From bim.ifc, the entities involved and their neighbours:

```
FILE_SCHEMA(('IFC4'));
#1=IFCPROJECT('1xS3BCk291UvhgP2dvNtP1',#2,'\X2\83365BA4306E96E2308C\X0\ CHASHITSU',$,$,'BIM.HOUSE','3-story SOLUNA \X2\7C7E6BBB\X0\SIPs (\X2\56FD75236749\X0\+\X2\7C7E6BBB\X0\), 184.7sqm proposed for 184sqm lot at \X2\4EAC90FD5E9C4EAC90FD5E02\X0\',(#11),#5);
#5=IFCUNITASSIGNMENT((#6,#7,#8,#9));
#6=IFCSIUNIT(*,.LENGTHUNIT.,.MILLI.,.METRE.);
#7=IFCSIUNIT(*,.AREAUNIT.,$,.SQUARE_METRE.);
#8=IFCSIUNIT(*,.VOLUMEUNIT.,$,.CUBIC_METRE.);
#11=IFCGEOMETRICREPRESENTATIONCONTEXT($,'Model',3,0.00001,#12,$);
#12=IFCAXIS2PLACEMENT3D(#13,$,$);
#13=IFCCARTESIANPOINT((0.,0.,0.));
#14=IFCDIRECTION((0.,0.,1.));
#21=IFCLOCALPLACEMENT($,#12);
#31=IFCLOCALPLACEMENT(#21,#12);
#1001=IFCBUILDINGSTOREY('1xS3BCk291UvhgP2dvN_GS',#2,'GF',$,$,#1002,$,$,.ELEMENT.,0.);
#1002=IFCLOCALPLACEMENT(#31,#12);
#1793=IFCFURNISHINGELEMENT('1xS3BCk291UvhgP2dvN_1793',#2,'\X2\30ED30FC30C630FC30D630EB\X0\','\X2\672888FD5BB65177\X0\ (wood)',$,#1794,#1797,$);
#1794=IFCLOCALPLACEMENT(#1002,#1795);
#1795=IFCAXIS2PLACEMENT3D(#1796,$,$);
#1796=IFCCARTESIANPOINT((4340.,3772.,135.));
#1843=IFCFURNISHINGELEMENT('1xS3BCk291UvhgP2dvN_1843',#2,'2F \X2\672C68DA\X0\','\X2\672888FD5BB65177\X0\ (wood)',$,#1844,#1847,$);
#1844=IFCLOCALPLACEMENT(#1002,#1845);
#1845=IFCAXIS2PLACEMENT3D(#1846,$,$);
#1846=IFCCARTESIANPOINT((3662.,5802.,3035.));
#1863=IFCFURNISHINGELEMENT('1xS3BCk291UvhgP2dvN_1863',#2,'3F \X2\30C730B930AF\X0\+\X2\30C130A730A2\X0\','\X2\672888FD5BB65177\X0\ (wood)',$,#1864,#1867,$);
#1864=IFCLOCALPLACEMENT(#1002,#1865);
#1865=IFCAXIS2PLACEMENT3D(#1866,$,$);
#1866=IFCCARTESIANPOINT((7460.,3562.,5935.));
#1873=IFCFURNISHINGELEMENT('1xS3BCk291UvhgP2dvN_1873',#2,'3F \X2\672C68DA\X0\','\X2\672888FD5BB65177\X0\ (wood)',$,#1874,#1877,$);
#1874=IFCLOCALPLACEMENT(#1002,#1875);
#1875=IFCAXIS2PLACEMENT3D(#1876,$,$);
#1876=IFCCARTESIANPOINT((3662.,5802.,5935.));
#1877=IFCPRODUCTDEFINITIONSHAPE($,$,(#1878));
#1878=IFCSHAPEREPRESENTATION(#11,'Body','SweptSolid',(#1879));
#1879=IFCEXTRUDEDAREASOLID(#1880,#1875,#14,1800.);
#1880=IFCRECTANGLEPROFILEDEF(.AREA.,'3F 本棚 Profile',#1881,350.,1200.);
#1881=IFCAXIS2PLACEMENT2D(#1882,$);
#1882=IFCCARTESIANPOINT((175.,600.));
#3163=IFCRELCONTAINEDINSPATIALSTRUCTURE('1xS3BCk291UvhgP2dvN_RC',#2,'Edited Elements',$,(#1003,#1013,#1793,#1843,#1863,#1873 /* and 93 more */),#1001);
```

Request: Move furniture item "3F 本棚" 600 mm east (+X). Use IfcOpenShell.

```python
import ifcopenshell
import ifcopenshell.api.geometry
import ifcopenshell.util.placement

model = ifcopenshell.open("bim.ifc")

item = model.by_guid("1xS3BCk291UvhgP2dvN_1873")
matrix = ifcopenshell.util.placement.get_local_placement(item.ObjectPlacement)
matrix[0, 3] += 600.0
ifcopenshell.api.geometry.edit_object_placement(model, product=item, matrix=matrix, is_si=False)

print(ifcopenshell.util.placement.get_local_placement(item.ObjectPlacement).round(3) + 0.0)

model.write("bim-out.ifc")
```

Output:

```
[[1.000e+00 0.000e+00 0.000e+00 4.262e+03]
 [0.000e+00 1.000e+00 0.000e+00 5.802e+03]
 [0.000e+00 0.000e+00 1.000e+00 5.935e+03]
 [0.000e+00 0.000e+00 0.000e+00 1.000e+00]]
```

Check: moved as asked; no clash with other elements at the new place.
